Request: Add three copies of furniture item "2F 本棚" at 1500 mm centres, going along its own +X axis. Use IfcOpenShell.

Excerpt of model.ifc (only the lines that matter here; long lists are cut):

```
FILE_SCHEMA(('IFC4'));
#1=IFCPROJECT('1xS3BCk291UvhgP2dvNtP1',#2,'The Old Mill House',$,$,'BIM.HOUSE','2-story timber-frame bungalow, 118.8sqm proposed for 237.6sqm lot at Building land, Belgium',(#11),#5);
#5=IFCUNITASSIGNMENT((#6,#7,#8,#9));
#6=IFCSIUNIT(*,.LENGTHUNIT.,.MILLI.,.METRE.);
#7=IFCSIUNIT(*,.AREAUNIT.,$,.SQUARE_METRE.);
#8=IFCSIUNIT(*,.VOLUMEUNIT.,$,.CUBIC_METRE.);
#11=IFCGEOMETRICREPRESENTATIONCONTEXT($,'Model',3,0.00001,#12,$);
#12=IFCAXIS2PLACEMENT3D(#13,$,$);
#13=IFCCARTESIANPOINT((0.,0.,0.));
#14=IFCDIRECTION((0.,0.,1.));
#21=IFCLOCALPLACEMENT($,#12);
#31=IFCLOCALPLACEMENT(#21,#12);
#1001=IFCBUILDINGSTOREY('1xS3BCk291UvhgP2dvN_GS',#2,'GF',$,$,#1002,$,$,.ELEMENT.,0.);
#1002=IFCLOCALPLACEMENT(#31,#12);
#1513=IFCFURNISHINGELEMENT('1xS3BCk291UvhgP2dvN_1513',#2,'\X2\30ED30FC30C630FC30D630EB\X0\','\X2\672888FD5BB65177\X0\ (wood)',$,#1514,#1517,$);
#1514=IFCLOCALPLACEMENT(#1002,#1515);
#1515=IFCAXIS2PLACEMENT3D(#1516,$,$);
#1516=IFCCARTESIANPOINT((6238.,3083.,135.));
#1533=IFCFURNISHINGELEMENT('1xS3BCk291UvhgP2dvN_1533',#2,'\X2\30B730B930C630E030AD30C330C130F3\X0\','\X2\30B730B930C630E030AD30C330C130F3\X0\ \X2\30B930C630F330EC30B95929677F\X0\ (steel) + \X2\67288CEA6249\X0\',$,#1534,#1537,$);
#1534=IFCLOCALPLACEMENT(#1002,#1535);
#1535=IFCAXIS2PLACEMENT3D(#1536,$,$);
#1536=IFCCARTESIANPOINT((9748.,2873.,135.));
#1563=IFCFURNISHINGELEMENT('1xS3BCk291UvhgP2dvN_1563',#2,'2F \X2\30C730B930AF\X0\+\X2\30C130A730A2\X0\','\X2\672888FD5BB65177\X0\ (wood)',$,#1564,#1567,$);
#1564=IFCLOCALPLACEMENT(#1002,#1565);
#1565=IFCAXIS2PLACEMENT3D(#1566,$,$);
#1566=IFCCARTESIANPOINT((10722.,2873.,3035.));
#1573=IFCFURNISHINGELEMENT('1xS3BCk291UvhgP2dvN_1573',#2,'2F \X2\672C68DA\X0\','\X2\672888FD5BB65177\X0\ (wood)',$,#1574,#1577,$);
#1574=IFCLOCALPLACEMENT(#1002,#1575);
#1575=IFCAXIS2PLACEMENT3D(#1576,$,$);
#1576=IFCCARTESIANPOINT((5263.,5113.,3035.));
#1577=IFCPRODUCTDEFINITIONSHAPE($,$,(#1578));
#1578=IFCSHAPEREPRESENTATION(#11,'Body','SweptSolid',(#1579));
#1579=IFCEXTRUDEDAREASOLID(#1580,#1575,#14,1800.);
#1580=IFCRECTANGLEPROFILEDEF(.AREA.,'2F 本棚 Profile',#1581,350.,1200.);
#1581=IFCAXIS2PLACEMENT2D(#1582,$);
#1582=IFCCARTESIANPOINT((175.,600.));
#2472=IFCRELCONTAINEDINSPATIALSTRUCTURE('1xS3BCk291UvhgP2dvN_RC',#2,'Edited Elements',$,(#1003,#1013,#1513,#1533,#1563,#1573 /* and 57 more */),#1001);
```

```python
import ifcopenshell
import ifcopenshell.api.geometry
import ifcopenshell.api.root
import ifcopenshell.util.element
import ifcopenshell.util.placement

model = ifcopenshell.open("model.ifc")


def reuse_history(source, copy):
    """copy_class also copies each property set's owner history, people and application; keep the originals."""
    for rel in copy.IsDefinedBy:
        if rel.is_a("IfcRelDefinesByProperties") and (history := rel.RelatingPropertyDefinition.OwnerHistory):
            rel.RelatingPropertyDefinition.OwnerHistory = source.OwnerHistory
            ifcopenshell.util.element.remove_deep2(model, history)


source = model.by_guid("1xS3BCk291UvhgP2dvN_1573")
base = ifcopenshell.util.placement.get_local_placement(source.ObjectPlacement)
step = base[:3, 0] * 1500.0

for i in range(1, 4):
    copy = ifcopenshell.api.root.copy_class(model, product=source)
    copy.Representation = ifcopenshell.util.element.copy_deep(
        model, source.Representation, exclude=["IfcGeometricRepresentationContext", "IfcRepresentationMap"]
    )
    reuse_history(source, copy)
    matrix = base.copy()
    matrix[:3, 3] += i * step
    print("added at", matrix[:3, 3].round(3) + 0.0)
    ifcopenshell.api.geometry.edit_object_placement(model, product=copy, matrix=matrix, is_si=False)

model.write("model-out.ifc")
```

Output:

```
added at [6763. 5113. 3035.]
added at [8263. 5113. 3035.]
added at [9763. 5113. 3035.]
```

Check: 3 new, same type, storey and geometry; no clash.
